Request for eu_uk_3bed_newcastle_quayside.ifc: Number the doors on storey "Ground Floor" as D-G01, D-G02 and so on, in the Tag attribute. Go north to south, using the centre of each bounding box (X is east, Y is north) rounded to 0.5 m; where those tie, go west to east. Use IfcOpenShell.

First a look at what the model holds.

```python
import ifcopenshell
import ifcopenshell.util.element
import ifcopenshell.util.placement

model = ifcopenshell.open("eu_uk_3bed_newcastle_quayside.ifc")
print(model.schema)
storey = next(s for s in model.by_type("IfcBuildingStorey") if s.Name == "Ground Floor")
doors = [e for e in ifcopenshell.util.element.get_decomposition(storey) if e.is_a("IfcDoor")]
for e in sorted(doors, key=lambda e: e.id()):
    origin = ifcopenshell.util.placement.get_local_placement(e.ObjectPlacement)[:3, 3]
    print(e.id(), e.Tag, e.Name, origin.round(2) + 0.0, sep=" | ")
```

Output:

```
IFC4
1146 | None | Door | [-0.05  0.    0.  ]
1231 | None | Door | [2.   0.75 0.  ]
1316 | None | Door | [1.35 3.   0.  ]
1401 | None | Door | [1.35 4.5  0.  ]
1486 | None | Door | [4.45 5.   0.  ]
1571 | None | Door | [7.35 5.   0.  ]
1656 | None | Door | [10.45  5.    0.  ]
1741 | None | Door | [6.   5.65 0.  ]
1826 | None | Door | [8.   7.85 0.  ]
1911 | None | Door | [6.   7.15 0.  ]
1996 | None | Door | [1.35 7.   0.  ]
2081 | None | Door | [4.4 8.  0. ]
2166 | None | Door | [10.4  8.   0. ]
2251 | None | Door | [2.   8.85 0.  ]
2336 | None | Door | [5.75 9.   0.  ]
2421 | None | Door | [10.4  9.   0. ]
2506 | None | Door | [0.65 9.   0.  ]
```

```python
import ifcopenshell
import ifcopenshell.geom
import ifcopenshell.util.element
import ifcopenshell.util.shape

model = ifcopenshell.open("eu_uk_3bed_newcastle_quayside.ifc")
settings = ifcopenshell.geom.settings()
settings.set("use-world-coords", True)


def centre(element):
    shape = ifcopenshell.geom.create_shape(settings, element)
    return ifcopenshell.util.shape.get_bbox_centroid(shape.geometry)


storey = next(s for s in model.by_type("IfcBuildingStorey") if s.Name == "Ground Floor")
doors = [e for e in ifcopenshell.util.element.get_decomposition(storey) if e.is_a("IfcDoor")]

# Insertion points can sit at a corner or the storey origin, so sort by the geometry (in metres).
centres = {e: centre(e) for e in doors}
doors.sort(key=lambda e: (-round(centres[e][1] / 0.5), centres[e][0]))

for i, e in enumerate(doors, start=1):
    number = f"D-G{i:02d}"
    e.Tag = number
    print(e.id(), number)

model.write("eu_uk_3bed_newcastle_quayside_v2.ifc")
```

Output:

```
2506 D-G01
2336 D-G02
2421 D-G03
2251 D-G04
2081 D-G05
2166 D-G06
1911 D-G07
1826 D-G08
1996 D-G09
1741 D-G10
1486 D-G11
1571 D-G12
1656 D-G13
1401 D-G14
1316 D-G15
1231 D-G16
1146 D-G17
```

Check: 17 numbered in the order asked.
